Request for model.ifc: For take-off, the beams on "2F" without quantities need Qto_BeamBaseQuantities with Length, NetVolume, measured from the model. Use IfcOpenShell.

First a look at what the model holds.

```python
import ifcopenshell
import ifcopenshell.util.element
import ifcopenshell.util.unit

model = ifcopenshell.open("model.ifc")
print(model.schema)
for unit_type in ("LENGTHUNIT", "AREAUNIT", "VOLUMEUNIT"):
    print(unit_type, ifcopenshell.util.unit.calculate_unit_scale(model, unit_type))
storey = next(s for s in model.by_type("IfcBuildingStorey") if s.Name == "2F")
beams = [e for e in ifcopenshell.util.element.get_decomposition(storey) if e.is_a("IfcBeam")]
for e in sorted(beams, key=lambda e: e.id()):
    print(e.id(), e.is_a(), e.Name, list(ifcopenshell.util.element.get_psets(e, qtos_only=True)), sep=" | ")
```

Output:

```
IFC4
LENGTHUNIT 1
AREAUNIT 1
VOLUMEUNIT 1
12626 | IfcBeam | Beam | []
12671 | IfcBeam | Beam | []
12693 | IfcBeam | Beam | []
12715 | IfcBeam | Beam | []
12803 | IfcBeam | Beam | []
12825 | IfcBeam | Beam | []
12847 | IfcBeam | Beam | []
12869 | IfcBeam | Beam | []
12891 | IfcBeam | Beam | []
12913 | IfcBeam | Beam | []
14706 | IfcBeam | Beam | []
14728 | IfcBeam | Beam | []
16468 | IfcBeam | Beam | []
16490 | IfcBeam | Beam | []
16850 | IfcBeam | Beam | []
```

```python
import ifcopenshell
import ifcopenshell.api.pset
import ifcopenshell.geom
import ifcopenshell.util.element
import ifcopenshell.util.shape
import ifcopenshell.util.unit

model = ifcopenshell.open("model.ifc")
unit_scale = ifcopenshell.util.unit.calculate_unit_scale(model)
volume_scale = ifcopenshell.util.unit.calculate_unit_scale(model, "VOLUMEUNIT")
settings = ifcopenshell.geom.settings()

storey = next(s for s in model.by_type("IfcBuildingStorey") if s.Name == "2F")
beams = [e for e in ifcopenshell.util.element.get_decomposition(storey) if e.is_a("IfcBeam")]

for e in sorted(beams, key=lambda e: e.id()):
    if ifcopenshell.util.element.get_psets(e, qtos_only=True, should_inherit=False):
        continue
    # Geometry comes back in metres, in the element's own axes.
    shape = ifcopenshell.geom.create_shape(settings, e)
    values = {
        "Length": ifcopenshell.util.shape.get_max_xyz(shape.geometry) / unit_scale,
        "NetVolume": ifcopenshell.util.shape.get_volume(shape.geometry) / volume_scale,
    }
    qto = ifcopenshell.api.pset.add_qto(model, product=e, name="Qto_BeamBaseQuantities")
    ifcopenshell.api.pset.edit_qto(model, qto=qto, properties=values)
    print(e.id(), {k: round(v, 3) for k, v in values.items()})

model.write("model_v2.ifc")
```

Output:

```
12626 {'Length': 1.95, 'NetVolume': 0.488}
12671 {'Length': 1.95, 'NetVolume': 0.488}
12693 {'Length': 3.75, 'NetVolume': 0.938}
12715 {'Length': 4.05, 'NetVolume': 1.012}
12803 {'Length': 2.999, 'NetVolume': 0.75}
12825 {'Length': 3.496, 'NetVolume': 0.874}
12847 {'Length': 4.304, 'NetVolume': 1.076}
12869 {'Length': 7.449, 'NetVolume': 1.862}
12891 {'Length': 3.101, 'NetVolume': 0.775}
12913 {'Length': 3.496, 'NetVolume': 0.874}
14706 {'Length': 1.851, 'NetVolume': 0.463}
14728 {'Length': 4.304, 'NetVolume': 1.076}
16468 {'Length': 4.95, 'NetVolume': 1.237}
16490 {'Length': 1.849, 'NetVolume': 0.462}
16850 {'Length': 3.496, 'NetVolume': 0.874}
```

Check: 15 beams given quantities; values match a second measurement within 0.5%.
